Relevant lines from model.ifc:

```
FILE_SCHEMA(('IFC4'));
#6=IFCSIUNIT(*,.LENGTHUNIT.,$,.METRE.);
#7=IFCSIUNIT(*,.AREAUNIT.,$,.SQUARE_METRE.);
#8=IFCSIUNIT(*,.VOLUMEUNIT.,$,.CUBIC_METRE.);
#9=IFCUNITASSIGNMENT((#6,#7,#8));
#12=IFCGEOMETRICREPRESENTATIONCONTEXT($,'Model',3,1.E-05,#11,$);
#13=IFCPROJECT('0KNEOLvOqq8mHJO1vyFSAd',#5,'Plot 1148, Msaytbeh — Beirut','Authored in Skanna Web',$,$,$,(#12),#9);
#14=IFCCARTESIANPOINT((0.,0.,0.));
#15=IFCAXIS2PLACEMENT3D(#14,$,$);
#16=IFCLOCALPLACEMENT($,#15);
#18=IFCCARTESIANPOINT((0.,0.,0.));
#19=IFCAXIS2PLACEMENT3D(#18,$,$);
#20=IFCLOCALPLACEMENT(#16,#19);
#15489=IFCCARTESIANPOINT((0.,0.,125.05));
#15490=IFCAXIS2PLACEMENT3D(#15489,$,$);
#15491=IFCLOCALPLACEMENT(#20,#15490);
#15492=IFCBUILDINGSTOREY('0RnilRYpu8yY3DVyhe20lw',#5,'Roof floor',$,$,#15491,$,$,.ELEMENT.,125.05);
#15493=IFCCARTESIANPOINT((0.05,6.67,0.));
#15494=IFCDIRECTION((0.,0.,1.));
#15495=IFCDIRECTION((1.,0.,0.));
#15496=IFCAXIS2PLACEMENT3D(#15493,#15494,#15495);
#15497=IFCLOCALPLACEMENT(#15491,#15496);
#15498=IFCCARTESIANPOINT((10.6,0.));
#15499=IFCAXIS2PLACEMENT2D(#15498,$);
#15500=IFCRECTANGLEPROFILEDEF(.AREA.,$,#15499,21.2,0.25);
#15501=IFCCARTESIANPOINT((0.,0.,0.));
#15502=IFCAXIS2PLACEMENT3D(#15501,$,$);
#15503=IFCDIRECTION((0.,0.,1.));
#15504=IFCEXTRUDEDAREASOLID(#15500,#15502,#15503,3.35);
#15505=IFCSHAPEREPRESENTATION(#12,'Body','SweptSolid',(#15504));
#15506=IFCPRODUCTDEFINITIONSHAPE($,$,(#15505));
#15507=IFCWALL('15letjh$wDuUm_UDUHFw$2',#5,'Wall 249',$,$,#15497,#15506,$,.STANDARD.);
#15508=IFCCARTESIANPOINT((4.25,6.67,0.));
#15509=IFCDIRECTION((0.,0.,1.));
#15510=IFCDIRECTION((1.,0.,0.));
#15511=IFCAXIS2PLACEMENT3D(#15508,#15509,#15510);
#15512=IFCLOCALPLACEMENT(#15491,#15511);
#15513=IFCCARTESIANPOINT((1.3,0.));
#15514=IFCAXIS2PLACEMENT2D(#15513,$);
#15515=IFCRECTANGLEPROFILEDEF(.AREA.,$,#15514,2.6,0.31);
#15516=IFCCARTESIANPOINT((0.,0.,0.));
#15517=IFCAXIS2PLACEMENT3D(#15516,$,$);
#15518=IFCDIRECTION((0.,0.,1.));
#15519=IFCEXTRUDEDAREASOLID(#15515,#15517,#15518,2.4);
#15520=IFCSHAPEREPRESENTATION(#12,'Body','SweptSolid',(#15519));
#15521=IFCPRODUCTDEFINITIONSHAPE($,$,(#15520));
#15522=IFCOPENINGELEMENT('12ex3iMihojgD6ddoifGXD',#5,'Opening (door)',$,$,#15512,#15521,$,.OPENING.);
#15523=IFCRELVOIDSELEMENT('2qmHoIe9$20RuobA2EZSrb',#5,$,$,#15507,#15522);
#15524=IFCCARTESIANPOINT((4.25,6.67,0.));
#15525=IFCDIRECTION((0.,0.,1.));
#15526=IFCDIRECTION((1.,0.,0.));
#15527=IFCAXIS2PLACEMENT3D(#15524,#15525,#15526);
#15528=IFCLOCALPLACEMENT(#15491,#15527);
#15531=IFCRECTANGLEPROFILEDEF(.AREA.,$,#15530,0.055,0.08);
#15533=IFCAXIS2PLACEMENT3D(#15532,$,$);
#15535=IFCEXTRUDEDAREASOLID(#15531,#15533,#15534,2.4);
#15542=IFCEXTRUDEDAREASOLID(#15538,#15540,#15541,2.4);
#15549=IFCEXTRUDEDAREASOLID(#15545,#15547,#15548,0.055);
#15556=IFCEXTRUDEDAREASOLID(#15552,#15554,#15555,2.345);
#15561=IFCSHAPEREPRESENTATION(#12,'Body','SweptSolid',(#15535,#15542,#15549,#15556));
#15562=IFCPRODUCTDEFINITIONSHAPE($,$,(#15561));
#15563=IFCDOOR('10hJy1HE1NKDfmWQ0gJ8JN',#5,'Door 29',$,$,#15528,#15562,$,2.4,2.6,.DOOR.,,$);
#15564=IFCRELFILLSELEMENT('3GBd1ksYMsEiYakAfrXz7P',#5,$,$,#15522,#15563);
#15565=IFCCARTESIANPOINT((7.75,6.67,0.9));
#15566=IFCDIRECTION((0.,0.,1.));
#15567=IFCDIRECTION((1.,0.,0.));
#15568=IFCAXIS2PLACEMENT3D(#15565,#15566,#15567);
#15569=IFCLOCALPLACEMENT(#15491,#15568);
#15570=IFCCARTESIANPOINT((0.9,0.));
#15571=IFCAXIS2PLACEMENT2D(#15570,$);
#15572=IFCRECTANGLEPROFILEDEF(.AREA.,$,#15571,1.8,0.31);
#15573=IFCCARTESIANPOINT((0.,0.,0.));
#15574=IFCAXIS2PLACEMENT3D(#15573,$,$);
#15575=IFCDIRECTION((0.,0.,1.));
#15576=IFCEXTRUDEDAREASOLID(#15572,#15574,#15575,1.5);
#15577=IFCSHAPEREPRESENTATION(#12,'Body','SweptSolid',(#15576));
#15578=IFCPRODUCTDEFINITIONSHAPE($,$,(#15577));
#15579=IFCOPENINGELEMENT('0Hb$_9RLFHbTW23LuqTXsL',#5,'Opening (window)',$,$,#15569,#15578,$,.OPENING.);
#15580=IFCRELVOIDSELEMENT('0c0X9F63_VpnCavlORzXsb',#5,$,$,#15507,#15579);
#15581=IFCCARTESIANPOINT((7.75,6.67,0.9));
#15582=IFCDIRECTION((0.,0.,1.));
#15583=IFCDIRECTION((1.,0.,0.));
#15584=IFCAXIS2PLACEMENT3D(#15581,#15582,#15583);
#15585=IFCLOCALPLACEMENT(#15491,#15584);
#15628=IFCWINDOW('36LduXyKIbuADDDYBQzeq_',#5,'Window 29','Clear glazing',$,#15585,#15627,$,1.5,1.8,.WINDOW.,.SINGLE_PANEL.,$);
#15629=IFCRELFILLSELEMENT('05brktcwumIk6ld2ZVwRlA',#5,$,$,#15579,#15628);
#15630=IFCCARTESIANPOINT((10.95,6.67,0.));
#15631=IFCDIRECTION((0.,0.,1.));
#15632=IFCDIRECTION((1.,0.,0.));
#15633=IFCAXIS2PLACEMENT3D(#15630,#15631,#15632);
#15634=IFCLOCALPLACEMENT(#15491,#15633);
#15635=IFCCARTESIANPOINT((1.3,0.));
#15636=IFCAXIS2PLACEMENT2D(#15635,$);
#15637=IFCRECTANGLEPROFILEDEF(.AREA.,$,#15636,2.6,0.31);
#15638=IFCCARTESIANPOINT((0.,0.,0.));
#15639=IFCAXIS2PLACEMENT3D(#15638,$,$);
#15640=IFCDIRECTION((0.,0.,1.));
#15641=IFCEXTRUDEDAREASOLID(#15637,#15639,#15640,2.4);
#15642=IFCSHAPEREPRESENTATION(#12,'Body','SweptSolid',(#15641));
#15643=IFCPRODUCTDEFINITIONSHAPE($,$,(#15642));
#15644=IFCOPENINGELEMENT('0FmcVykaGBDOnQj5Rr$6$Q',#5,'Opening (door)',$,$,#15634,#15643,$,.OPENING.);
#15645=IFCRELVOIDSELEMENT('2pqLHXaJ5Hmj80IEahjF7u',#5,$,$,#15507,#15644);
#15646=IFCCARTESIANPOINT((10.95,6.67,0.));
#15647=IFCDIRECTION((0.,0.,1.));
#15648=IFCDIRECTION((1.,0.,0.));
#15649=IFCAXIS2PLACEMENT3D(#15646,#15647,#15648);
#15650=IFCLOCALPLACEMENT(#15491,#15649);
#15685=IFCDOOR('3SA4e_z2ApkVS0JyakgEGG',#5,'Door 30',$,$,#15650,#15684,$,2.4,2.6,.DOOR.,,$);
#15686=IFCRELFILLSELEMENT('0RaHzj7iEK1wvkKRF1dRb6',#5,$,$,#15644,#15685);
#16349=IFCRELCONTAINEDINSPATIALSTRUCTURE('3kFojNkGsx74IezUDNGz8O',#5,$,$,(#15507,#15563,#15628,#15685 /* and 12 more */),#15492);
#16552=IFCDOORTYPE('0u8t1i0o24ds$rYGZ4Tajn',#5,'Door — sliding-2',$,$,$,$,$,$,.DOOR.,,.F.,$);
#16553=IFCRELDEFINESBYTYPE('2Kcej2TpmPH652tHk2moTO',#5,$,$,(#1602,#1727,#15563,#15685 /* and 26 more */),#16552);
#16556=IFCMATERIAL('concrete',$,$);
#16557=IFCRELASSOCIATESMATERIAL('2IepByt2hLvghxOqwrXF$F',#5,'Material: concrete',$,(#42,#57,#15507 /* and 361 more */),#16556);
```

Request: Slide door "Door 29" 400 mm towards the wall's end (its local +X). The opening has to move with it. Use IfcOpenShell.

```python
import ifcopenshell
import ifcopenshell.api.geometry
import ifcopenshell.util.placement

model = ifcopenshell.open("model.ifc")

door = model.by_guid("10hJy1HE1NKDfmWQ0gJ8JN")
opening = door.FillsVoids[0].RelatingOpeningElement
wall = opening.VoidsElements[0].RelatingBuildingElement

wall_matrix = ifcopenshell.util.placement.get_local_placement(wall.ObjectPlacement)
shift = wall_matrix[:3, 0] * 0.4
before = ifcopenshell.util.placement.get_local_placement(door.ObjectPlacement)[:3, 3].copy()

# The door is not placed relative to its opening, so move both.
for product in (opening, door):
    matrix = ifcopenshell.util.placement.get_local_placement(product.ObjectPlacement)
    matrix[:3, 3] += shift
    ifcopenshell.api.geometry.edit_object_placement(model, product=product, matrix=matrix, is_si=False)

after = ifcopenshell.util.placement.get_local_placement(door.ObjectPlacement)[:3, 3]
print("door moved by", (after - before).round(3) + 0.0)

model.write("model_v2.ifc")
```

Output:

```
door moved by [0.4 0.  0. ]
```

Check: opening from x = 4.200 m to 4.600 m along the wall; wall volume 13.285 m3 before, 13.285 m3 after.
